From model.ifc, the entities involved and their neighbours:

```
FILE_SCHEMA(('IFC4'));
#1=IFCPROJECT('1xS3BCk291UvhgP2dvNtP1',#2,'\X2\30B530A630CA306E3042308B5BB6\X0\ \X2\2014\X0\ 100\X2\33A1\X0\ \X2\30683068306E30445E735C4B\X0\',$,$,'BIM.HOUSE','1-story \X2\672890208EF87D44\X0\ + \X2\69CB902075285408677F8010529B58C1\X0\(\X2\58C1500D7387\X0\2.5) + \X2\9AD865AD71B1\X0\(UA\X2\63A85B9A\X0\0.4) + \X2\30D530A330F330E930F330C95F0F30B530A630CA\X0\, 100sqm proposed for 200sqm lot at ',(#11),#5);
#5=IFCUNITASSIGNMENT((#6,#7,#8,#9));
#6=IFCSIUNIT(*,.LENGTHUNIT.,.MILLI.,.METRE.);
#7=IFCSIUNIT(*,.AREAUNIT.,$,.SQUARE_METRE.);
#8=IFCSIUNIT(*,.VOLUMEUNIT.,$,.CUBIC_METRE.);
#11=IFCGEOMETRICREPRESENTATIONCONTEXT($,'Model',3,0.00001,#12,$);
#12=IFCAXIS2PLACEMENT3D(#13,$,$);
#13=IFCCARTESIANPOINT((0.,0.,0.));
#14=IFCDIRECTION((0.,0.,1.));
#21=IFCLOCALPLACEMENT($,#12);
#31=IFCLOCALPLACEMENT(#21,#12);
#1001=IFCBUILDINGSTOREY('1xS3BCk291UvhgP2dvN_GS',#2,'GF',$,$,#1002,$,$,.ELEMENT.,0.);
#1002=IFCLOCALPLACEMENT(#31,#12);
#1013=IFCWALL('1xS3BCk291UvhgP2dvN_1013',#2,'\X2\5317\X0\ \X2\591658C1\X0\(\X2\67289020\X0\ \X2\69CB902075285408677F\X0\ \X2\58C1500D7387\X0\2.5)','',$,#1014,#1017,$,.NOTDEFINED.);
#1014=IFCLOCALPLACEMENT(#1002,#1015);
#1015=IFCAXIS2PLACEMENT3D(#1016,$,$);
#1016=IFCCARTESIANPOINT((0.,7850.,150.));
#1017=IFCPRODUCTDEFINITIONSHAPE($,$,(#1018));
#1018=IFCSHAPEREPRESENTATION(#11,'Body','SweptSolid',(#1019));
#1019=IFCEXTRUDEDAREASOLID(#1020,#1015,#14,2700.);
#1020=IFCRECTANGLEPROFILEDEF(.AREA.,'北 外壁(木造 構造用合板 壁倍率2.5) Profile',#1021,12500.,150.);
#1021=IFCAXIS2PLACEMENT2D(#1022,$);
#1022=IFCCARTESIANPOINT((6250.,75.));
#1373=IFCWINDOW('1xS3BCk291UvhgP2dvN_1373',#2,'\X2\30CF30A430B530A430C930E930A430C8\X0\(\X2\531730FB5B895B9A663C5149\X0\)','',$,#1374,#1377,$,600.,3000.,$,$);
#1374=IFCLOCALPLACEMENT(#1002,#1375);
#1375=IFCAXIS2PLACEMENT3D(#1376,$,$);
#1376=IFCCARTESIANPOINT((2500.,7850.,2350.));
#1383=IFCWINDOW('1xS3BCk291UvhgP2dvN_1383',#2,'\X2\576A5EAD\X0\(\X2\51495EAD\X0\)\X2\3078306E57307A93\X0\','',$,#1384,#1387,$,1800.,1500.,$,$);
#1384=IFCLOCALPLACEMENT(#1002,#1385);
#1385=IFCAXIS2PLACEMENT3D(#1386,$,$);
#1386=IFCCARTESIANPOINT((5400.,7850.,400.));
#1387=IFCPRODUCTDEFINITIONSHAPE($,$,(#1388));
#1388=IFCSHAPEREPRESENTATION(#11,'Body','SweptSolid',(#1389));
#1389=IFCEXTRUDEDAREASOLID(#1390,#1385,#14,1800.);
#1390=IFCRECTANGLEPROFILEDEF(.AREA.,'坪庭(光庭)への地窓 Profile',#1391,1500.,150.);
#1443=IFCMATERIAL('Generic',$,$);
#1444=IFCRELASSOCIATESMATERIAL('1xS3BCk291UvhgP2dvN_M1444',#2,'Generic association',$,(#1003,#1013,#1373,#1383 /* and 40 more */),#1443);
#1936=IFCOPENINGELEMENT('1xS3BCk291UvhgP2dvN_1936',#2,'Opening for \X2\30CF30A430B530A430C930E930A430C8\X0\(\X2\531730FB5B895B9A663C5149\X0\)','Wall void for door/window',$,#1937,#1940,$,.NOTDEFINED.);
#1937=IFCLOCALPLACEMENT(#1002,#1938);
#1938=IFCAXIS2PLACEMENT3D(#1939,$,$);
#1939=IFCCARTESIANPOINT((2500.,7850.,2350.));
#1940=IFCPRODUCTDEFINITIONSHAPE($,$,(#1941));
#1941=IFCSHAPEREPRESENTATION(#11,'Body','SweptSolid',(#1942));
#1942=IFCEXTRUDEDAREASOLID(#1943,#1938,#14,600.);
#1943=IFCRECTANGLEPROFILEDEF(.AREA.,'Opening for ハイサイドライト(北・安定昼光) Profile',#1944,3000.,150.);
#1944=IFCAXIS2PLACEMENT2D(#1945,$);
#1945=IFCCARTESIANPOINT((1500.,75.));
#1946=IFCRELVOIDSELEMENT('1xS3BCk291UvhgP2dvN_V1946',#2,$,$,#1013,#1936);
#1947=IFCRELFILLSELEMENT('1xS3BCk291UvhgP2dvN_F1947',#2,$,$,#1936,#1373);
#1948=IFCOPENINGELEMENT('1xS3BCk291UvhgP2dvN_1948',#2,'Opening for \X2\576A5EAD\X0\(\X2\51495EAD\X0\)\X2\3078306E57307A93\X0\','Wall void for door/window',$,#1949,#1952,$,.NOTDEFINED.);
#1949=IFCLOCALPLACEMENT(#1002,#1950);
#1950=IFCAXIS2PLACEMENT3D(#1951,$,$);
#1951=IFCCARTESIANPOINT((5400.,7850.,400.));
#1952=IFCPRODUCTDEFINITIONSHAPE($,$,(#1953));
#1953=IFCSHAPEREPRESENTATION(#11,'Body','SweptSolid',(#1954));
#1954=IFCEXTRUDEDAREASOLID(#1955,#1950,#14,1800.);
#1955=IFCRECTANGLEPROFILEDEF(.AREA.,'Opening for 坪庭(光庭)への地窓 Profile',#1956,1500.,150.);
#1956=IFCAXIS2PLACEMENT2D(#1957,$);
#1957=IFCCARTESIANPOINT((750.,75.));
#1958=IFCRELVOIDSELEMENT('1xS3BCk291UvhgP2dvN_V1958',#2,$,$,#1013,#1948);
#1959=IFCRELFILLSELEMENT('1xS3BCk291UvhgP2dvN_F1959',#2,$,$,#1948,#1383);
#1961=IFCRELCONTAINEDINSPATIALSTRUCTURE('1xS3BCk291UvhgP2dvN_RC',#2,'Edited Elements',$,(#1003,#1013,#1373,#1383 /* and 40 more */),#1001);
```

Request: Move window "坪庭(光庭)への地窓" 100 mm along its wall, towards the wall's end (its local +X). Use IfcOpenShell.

```python
import ifcopenshell
import ifcopenshell.api.geometry
import ifcopenshell.util.placement
import ifcopenshell.util.unit

model = ifcopenshell.open("model.ifc")
unit_scale = ifcopenshell.util.unit.calculate_unit_scale(model)

window = model.by_guid("1xS3BCk291UvhgP2dvN_1383")
opening = window.FillsVoids[0].RelatingOpeningElement
wall = opening.VoidsElements[0].RelatingBuildingElement

wall_matrix = ifcopenshell.util.placement.get_local_placement(wall.ObjectPlacement)
shift = wall_matrix[:3, 0] * 0.1 / unit_scale
before = ifcopenshell.util.placement.get_local_placement(window.ObjectPlacement)[:3, 3].copy()

# The window is not placed relative to its opening, so move both.
for product in (opening, window):
    matrix = ifcopenshell.util.placement.get_local_placement(product.ObjectPlacement)
    matrix[:3, 3] += shift
    ifcopenshell.api.geometry.edit_object_placement(model, product=product, matrix=matrix, is_si=False)

after = ifcopenshell.util.placement.get_local_placement(window.ObjectPlacement)[:3, 3]
print("window moved by", (after - before).round(3) + 0.0)

model.write("model_rev.ifc")
```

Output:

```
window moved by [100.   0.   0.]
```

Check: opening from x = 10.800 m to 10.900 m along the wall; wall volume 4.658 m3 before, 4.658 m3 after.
